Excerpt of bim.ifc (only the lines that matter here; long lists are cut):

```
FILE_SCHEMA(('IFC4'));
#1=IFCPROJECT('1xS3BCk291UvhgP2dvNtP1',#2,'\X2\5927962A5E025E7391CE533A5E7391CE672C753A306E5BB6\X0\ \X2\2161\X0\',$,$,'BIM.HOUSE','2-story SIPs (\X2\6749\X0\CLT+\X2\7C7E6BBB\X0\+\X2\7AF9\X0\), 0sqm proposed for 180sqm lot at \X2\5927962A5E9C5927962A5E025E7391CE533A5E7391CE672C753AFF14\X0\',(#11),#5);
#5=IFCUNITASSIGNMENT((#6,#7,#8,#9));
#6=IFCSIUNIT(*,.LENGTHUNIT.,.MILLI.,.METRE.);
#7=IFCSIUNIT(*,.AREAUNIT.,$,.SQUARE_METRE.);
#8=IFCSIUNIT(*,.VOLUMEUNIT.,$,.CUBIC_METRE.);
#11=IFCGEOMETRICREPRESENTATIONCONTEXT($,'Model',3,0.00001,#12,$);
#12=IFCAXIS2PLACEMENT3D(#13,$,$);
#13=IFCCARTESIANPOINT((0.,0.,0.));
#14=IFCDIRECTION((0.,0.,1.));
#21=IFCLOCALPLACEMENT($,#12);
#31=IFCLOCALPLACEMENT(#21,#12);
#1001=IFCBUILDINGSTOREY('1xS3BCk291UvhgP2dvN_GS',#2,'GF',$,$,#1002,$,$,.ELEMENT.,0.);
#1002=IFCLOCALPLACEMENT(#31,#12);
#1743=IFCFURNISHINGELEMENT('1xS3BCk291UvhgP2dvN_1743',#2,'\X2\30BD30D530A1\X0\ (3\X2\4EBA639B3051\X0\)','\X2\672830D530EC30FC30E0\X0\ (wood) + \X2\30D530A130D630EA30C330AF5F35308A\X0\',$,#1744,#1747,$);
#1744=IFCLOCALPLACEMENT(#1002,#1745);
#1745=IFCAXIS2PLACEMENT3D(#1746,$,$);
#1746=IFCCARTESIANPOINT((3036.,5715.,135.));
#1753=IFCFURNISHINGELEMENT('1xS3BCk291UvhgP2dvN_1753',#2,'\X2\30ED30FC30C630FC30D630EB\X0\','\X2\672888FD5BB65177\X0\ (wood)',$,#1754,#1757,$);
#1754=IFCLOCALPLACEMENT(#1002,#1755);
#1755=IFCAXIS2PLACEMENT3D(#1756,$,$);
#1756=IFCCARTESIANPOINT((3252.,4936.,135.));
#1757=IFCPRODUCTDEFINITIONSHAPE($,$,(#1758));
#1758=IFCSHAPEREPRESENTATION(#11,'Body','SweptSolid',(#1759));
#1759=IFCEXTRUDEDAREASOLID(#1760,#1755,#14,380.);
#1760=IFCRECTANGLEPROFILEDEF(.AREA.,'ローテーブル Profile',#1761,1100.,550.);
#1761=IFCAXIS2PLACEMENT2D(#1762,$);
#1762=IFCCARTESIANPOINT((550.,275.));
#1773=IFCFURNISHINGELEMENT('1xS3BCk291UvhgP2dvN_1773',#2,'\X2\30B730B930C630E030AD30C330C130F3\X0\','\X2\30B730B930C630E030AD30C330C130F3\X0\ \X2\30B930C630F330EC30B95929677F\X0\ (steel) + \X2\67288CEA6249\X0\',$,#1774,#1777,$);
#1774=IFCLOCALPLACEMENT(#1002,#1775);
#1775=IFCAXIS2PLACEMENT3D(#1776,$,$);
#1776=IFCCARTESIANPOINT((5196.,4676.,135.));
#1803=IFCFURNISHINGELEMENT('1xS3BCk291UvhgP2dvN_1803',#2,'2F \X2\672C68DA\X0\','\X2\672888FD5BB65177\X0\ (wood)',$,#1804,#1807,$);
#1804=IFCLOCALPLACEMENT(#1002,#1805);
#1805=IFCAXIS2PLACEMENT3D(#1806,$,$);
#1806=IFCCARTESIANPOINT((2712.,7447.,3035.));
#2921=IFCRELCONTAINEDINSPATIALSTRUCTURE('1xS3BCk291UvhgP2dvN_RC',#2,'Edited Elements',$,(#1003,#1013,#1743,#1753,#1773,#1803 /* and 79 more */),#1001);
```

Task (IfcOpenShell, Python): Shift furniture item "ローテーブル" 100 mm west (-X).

```python
import ifcopenshell
import ifcopenshell.api.geometry
import ifcopenshell.util.placement
import ifcopenshell.util.unit

model = ifcopenshell.open("bim.ifc")
unit_scale = ifcopenshell.util.unit.calculate_unit_scale(model)

item = model.by_guid("1xS3BCk291UvhgP2dvN_1753")
matrix = ifcopenshell.util.placement.get_local_placement(item.ObjectPlacement)
matrix[0, 3] -= 0.1 / unit_scale
ifcopenshell.api.geometry.edit_object_placement(model, product=item, matrix=matrix, is_si=False)

print(ifcopenshell.util.placement.get_local_placement(item.ObjectPlacement).round(3) + 0.0)

model.write("bim_rev.ifc")
```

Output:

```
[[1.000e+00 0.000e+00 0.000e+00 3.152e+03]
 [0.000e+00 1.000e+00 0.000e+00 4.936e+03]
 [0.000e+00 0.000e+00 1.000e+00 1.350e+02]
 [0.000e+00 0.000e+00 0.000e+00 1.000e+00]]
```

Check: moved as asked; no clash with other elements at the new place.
